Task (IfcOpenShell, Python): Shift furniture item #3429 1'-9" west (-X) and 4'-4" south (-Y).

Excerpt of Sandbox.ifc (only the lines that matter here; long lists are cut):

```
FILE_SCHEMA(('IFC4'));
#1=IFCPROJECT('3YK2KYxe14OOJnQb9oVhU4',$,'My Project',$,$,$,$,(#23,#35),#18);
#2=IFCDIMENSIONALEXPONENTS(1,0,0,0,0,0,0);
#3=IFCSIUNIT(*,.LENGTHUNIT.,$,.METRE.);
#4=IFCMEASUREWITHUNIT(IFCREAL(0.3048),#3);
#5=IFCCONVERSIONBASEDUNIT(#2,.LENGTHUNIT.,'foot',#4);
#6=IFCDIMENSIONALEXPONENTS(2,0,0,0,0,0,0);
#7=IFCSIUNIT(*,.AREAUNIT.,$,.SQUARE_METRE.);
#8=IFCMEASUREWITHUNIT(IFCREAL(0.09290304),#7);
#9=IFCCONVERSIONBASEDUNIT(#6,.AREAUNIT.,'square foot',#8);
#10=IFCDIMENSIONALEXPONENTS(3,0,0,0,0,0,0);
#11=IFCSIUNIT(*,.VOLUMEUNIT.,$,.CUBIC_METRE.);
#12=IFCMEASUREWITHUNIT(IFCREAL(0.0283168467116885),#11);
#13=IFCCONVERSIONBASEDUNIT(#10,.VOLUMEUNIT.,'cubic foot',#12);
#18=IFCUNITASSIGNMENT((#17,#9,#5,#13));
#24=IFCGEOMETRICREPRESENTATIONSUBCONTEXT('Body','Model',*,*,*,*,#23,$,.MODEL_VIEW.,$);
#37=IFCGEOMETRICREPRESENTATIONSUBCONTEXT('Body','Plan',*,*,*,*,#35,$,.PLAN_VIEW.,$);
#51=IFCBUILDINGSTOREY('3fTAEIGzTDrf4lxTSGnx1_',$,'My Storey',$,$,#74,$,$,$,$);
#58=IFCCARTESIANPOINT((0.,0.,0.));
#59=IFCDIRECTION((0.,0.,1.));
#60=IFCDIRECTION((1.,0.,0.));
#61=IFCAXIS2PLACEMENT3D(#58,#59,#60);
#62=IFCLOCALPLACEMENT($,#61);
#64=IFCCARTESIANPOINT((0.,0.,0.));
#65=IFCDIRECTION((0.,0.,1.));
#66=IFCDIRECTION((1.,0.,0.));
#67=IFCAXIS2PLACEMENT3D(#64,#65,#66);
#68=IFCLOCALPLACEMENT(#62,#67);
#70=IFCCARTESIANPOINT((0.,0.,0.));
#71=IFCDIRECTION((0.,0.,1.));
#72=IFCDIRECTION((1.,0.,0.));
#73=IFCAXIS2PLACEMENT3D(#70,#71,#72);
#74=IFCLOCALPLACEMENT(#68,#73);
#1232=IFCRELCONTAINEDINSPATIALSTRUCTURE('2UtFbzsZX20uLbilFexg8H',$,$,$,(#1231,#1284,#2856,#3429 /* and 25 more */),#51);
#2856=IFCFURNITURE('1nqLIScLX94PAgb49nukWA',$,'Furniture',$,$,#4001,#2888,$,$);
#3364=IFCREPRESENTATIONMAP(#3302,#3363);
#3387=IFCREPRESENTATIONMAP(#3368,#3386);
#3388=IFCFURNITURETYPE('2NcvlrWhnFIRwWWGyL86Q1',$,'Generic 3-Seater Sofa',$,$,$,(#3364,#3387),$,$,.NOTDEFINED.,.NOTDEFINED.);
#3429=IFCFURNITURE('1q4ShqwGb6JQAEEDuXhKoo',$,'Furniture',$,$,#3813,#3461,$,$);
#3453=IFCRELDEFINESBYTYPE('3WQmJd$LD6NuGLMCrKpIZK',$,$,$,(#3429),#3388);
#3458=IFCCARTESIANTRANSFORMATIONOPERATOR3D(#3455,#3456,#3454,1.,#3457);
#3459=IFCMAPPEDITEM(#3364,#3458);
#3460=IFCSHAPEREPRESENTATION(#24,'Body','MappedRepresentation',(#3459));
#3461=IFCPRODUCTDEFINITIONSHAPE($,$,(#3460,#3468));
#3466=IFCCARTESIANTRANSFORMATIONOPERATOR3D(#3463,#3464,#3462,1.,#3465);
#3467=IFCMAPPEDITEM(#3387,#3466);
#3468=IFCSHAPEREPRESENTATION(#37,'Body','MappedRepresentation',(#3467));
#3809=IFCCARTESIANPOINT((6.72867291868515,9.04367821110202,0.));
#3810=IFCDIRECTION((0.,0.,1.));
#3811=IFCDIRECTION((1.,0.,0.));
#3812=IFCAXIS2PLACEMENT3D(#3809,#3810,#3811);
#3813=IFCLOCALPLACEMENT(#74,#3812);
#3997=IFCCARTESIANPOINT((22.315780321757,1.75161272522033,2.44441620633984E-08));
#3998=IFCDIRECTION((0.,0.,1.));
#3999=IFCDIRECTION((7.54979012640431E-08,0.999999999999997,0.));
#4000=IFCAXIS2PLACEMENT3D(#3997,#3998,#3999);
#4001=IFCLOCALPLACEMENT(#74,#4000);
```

```python
import ifcopenshell
import ifcopenshell.api.geometry
import ifcopenshell.util.placement
import ifcopenshell.util.unit

model = ifcopenshell.open("Sandbox.ifc")
unit_scale = ifcopenshell.util.unit.calculate_unit_scale(model)

item = model.by_id(3429)
matrix = ifcopenshell.util.placement.get_local_placement(item.ObjectPlacement)
matrix[0, 3] -= 21 * 0.0254 / unit_scale
matrix[1, 3] -= 52 * 0.0254 / unit_scale
ifcopenshell.api.geometry.edit_object_placement(model, product=item, matrix=matrix, is_si=False)

print(ifcopenshell.util.placement.get_local_placement(item.ObjectPlacement).round(3) + 0.0)

model.write("Sandbox_edited.ifc")
```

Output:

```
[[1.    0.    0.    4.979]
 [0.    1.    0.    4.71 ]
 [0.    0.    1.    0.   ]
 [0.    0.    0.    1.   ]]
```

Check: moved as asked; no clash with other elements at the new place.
